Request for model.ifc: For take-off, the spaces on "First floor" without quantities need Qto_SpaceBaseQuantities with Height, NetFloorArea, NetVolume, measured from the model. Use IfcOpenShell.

First a look at what the model holds.

```python
import ifcopenshell
import ifcopenshell.util.element
import ifcopenshell.util.unit

model = ifcopenshell.open("model.ifc")
print(model.schema)
for unit_type in ("LENGTHUNIT", "AREAUNIT", "VOLUMEUNIT"):
    print(unit_type, ifcopenshell.util.unit.calculate_unit_scale(model, unit_type))
storey = next(s for s in model.by_type("IfcBuildingStorey") if s.Name == "First floor")
spaces = [e for e in ifcopenshell.util.element.get_decomposition(storey) if e.is_a("IfcSpace")]
for e in sorted(spaces, key=lambda e: e.id()):
    print(e.id(), e.is_a(), e.Name, list(ifcopenshell.util.element.get_psets(e, qtos_only=True)), sep=" | ")
```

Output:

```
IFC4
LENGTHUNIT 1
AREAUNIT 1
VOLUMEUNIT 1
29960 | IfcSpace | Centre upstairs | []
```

```python
import ifcopenshell
import ifcopenshell.api.pset
import ifcopenshell.geom
import ifcopenshell.util.element
import ifcopenshell.util.shape
import ifcopenshell.util.unit

model = ifcopenshell.open("model.ifc")
unit_scale = ifcopenshell.util.unit.calculate_unit_scale(model)
area_scale = ifcopenshell.util.unit.calculate_unit_scale(model, "AREAUNIT")
volume_scale = ifcopenshell.util.unit.calculate_unit_scale(model, "VOLUMEUNIT")
settings = ifcopenshell.geom.settings()

storey = next(s for s in model.by_type("IfcBuildingStorey") if s.Name == "First floor")
spaces = [e for e in ifcopenshell.util.element.get_decomposition(storey) if e.is_a("IfcSpace")]

for e in sorted(spaces, key=lambda e: e.id()):
    if ifcopenshell.util.element.get_psets(e, qtos_only=True, should_inherit=False):
        continue
    # Geometry comes back in metres, in the element's own axes.
    shape = ifcopenshell.geom.create_shape(settings, e)
    values = {
        "Height": ifcopenshell.util.shape.get_z(shape.geometry) / unit_scale,
        "NetFloorArea": ifcopenshell.util.shape.get_footprint_area(shape.geometry) / area_scale,
        "NetVolume": ifcopenshell.util.shape.get_volume(shape.geometry) / volume_scale,
    }
    qto = ifcopenshell.api.pset.add_qto(model, product=e, name="Qto_SpaceBaseQuantities")
    ifcopenshell.api.pset.edit_qto(model, qto=qto, properties=values)
    print(e.id(), {k: round(v, 3) for k, v in values.items()})

model.write("model_rev.ifc")
```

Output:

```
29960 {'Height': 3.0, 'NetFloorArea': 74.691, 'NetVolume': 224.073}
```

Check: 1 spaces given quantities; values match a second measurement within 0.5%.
